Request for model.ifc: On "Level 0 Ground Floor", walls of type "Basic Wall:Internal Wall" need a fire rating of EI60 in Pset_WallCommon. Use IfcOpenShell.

First a look at what the model holds.

```python
import ifcopenshell
import ifcopenshell.util.element

model = ifcopenshell.open("model.ifc")
print(model.schema)
storey = next(s for s in model.by_type("IfcBuildingStorey") if s.Name == "Level 0 Ground Floor")
walls = [e for e in ifcopenshell.util.element.get_decomposition(storey) if e.is_a("IfcWall")]
seen = {}
for e in walls:
    element_type = ifcopenshell.util.element.get_type(e)
    key = (element_type.Name if element_type != e and element_type else None, ifcopenshell.util.element.get_pset(e, "Pset_WallCommon", "FireRating"))
    seen[key] = seen.get(key, 0) + 1
for (name, value), count in sorted(seen.items(), key=str):
    print(count, "x", name, "|", value)
```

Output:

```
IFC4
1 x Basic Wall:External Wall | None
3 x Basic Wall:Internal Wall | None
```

```python
import ifcopenshell
import ifcopenshell.api.pset
import ifcopenshell.util.element

model = ifcopenshell.open("model.ifc")

storey = next(s for s in model.by_type("IfcBuildingStorey") if s.Name == "Level 0 Ground Floor")
walls = [e for e in ifcopenshell.util.element.get_decomposition(storey) if e.is_a("IfcWall")]

count = 0
for e in walls:
    element_type = ifcopenshell.util.element.get_type(e)
    if element_type in (None, e) or element_type.Name != "Basic Wall:Internal Wall":
        continue
    # add_pset returns the element's existing set when there is one.
    pset = ifcopenshell.api.pset.add_pset(model, product=e, name="Pset_WallCommon")
    ifcopenshell.api.pset.edit_pset(model, pset=pset, properties={"FireRating": "EI60"})
    count += 1

print(count, "walls updated")

model.write("model-out.ifc")
```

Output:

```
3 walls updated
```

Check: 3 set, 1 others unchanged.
